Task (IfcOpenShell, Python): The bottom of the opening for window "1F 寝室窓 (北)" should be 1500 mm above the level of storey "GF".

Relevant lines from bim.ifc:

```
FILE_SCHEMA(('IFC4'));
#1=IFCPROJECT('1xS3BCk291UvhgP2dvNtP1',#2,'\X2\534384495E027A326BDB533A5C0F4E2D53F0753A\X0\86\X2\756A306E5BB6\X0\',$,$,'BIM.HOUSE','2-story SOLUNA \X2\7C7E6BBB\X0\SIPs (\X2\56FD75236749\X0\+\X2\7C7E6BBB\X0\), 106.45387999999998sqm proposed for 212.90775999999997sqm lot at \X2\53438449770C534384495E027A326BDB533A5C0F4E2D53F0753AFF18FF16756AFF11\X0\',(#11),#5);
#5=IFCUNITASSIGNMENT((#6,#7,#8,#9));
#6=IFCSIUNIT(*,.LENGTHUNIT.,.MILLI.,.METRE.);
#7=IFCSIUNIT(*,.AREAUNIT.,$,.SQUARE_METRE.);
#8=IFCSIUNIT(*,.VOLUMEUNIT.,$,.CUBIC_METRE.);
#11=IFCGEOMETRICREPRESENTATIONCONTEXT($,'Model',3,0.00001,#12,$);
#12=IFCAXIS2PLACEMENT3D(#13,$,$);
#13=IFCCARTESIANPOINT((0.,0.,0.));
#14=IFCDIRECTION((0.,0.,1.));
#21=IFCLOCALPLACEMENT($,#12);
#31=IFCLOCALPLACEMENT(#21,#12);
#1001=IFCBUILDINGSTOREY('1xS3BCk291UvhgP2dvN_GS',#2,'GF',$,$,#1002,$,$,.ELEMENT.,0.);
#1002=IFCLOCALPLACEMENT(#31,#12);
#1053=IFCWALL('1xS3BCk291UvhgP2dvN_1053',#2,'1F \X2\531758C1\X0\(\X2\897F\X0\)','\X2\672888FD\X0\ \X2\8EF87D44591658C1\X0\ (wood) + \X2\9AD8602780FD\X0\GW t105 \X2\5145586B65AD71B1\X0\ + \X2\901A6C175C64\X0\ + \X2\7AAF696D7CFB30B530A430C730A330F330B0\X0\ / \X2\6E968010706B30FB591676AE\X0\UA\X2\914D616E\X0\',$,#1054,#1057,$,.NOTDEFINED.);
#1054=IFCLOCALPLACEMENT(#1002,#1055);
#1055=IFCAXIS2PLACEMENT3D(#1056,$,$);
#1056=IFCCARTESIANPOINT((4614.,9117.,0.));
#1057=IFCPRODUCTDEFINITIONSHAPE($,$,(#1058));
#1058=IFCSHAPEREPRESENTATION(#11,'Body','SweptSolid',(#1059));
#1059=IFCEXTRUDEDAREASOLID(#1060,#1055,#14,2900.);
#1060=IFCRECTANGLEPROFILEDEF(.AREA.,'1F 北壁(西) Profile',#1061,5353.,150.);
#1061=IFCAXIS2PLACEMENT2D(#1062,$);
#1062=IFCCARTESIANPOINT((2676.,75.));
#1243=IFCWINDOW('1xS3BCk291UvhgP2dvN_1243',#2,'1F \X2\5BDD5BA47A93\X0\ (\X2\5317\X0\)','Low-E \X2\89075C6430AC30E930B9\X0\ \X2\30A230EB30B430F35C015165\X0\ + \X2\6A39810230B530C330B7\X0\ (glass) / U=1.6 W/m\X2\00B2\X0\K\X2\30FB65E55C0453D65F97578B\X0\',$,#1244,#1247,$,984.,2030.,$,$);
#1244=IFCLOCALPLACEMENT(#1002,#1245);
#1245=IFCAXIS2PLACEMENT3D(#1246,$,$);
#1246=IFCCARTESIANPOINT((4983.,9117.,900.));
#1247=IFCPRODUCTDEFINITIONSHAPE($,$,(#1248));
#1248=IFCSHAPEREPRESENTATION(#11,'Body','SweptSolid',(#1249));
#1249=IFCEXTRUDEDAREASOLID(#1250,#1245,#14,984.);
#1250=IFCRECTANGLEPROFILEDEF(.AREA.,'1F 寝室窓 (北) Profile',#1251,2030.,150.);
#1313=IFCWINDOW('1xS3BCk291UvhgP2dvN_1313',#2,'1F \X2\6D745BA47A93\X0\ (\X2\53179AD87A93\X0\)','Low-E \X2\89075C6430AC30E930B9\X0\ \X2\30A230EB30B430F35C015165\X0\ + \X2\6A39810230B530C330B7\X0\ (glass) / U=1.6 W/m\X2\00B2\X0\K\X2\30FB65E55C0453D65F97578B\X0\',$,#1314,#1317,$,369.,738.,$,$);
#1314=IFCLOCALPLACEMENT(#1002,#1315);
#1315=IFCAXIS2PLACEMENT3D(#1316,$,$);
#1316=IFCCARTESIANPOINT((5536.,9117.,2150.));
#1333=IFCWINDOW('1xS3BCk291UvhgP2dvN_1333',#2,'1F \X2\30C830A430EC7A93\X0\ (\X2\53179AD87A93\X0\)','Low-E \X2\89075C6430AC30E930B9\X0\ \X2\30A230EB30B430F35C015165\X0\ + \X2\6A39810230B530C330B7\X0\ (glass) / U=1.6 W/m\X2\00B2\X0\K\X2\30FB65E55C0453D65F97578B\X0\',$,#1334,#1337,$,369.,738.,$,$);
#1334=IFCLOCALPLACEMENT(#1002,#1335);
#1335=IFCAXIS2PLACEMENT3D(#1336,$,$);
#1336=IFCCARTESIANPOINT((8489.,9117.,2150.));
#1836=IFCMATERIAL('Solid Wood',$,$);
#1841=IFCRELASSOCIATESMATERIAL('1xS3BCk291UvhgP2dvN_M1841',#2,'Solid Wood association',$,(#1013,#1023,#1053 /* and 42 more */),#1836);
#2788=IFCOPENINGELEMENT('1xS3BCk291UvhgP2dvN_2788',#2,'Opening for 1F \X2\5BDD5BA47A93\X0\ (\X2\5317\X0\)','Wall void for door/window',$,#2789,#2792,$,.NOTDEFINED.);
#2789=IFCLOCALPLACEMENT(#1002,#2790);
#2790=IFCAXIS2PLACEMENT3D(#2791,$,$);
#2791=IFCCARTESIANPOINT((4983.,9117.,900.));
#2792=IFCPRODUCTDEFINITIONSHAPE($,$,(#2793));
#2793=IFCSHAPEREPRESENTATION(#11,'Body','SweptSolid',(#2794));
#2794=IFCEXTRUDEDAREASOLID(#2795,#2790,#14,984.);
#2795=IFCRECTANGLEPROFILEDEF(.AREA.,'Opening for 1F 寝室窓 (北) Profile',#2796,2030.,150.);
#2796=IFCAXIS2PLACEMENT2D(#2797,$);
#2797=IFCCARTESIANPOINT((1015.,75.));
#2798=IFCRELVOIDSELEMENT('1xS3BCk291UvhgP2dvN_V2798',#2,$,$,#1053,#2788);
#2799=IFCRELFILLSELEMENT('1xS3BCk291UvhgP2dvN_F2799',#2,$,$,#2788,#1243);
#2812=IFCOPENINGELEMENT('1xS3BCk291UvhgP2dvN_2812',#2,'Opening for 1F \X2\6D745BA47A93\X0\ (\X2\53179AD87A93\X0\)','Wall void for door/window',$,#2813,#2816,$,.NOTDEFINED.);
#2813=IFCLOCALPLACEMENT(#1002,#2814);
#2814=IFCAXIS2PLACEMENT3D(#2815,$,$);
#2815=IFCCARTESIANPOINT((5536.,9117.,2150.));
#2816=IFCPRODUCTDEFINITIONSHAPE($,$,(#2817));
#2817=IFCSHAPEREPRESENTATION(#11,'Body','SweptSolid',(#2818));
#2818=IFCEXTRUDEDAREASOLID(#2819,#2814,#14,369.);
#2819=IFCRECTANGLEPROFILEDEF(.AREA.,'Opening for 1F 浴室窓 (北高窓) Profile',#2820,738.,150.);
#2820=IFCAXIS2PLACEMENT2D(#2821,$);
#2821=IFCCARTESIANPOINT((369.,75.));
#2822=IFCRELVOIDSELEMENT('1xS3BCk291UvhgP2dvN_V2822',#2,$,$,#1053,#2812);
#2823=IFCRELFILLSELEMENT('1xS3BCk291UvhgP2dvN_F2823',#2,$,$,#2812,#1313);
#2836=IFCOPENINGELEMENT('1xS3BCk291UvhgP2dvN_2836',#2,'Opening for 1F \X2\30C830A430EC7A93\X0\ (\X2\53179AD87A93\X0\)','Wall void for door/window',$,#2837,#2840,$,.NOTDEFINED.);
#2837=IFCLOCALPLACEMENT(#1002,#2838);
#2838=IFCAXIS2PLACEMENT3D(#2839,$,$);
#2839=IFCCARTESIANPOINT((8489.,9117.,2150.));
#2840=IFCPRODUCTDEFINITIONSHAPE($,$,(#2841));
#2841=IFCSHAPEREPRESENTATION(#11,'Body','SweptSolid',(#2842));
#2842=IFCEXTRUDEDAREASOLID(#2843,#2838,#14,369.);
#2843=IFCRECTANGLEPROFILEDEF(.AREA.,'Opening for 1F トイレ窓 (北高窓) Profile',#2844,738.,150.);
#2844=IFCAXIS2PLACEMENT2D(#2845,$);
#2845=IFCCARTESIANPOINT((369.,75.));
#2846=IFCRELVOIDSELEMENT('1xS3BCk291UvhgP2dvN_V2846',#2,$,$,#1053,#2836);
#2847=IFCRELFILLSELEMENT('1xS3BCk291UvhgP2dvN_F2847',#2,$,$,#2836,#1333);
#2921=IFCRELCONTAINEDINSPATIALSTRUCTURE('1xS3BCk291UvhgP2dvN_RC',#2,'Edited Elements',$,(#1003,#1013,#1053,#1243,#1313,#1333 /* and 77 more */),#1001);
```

```python
import numpy as np
import ifcopenshell
import ifcopenshell.api.geometry
import ifcopenshell.geom
import ifcopenshell.util.element
import ifcopenshell.util.placement
import ifcopenshell.util.shape
import ifcopenshell.util.unit

model = ifcopenshell.open("bim.ifc")
unit_scale = ifcopenshell.util.unit.calculate_unit_scale(model)

window = model.by_guid("1xS3BCk291UvhgP2dvN_1243")
opening = window.FillsVoids[0].RelatingOpeningElement
storey = ifcopenshell.util.element.get_container(window, ifc_class="IfcBuildingStorey")
level = ifcopenshell.util.placement.get_local_placement(storey.ObjectPlacement)[2, 3]

# The opening's origin need not be at the sill, so measure its lowest point.
shape = ifcopenshell.geom.create_shape(ifcopenshell.geom.settings(), opening)
bottom = ifcopenshell.util.shape.get_shape_bottom_elevation(shape, shape.geometry) / unit_scale
dz = level + 1500.0 - bottom

shift = np.array([0.0, 0.0, dz])
# The window is not placed relative to its opening, so move both.
for product in (opening, window):
    matrix = ifcopenshell.util.placement.get_local_placement(product.ObjectPlacement)
    matrix[:3, 3] += shift
    ifcopenshell.api.geometry.edit_object_placement(model, product=product, matrix=matrix, is_si=False)

print(f"moved by {dz * unit_scale:+.3f} m")

model.write("bim_edited.ifc")
```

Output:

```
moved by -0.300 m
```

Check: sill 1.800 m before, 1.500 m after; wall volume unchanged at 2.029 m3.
